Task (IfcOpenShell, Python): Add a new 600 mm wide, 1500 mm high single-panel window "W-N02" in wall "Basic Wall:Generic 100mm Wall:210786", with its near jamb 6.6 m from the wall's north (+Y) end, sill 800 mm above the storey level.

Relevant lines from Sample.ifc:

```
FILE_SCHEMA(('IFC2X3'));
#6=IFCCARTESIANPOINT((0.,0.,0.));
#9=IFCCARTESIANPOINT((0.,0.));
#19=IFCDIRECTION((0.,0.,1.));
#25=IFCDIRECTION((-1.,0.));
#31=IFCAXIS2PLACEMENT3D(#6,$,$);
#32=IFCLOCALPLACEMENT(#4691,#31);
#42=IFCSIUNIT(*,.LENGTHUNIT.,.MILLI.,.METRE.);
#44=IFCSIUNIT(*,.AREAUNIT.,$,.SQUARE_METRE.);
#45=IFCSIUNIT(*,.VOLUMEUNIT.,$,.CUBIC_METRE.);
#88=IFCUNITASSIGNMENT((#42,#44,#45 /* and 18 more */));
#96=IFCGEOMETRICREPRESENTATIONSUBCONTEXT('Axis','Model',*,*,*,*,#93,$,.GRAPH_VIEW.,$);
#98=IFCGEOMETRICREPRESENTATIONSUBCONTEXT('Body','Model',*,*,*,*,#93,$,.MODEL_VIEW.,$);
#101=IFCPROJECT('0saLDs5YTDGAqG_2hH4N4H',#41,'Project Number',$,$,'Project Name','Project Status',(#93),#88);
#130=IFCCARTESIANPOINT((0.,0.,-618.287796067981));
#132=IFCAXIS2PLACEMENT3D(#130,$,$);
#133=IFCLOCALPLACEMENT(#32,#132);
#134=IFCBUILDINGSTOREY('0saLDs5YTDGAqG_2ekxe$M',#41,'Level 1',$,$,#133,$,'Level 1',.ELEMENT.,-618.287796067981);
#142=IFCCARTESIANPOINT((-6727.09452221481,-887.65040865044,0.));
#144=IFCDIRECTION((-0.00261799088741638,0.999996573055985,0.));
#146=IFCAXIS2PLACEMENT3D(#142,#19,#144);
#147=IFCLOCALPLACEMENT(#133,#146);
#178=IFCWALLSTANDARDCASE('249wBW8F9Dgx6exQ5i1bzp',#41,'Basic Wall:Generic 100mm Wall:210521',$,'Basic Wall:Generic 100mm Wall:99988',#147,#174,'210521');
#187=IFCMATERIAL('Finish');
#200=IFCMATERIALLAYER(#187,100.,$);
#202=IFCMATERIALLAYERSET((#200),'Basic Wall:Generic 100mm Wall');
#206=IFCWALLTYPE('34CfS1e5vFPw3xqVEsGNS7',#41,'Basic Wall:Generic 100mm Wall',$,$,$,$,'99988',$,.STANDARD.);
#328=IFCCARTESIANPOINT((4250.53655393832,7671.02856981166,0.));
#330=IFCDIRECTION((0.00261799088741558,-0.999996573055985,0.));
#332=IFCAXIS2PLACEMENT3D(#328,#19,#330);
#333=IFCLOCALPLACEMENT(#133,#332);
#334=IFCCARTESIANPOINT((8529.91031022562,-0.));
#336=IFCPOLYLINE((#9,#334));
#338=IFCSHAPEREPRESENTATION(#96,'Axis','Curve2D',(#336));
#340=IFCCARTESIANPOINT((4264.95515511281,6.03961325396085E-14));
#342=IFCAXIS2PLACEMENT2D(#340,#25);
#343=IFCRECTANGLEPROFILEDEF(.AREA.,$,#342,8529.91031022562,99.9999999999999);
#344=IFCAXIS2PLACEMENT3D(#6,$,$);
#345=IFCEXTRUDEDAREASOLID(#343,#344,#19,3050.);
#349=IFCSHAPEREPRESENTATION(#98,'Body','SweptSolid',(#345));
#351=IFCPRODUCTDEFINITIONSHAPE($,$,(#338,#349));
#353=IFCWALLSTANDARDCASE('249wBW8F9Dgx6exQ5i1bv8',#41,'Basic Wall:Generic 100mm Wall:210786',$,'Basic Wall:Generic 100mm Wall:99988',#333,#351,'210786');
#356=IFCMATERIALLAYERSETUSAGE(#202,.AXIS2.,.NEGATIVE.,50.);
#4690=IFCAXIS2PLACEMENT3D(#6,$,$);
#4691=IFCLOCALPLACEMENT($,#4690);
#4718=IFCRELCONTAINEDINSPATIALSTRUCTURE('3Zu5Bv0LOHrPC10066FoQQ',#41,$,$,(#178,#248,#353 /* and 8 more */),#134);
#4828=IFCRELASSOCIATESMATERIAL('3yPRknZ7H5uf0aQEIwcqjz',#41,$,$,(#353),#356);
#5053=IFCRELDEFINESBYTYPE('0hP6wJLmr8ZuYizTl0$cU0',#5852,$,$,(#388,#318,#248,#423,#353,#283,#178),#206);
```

```python
import numpy as np
import ifcopenshell
import ifcopenshell.api.feature
import ifcopenshell.api.geometry
import ifcopenshell.api.root
import ifcopenshell.api.spatial
import ifcopenshell.api.type
import ifcopenshell.geom
import ifcopenshell.util.element
import ifcopenshell.util.placement
import ifcopenshell.util.representation
import ifcopenshell.util.shape
import ifcopenshell.util.unit

model = ifcopenshell.open("Sample.ifc")
unit_scale = ifcopenshell.util.unit.calculate_unit_scale(model)
settings = ifcopenshell.geom.settings()


def volume(element):
    """Net volume in cubic metres, openings subtracted."""
    shape = ifcopenshell.geom.create_shape(settings, element)
    return ifcopenshell.util.shape.get_volume(shape.geometry)


wall = model.by_id(353)
storey = ifcopenshell.util.element.get_container(wall, ifc_class="IfcBuildingStorey")
context = ifcopenshell.util.representation.get_context(model, "Model", "Body", "MODEL_VIEW")
before = volume(wall)

width, height, from_end, sill = 0.6, 1.5, 6.6, 0.8  # metres

# The wall runs along its own X axis, and the end named is its -X end.
wall_shape = ifcopenshell.geom.create_shape(settings, wall)
x, y, z = ifcopenshell.util.shape.get_vertices(wall_shape.geometry).T
start = x.min() + from_end
face, thickness = float(y.min()), float(y.max() - y.min())
wall_matrix = ifcopenshell.util.placement.get_local_placement(wall.ObjectPlacement)
level = ifcopenshell.util.placement.get_local_placement(storey.ObjectPlacement)[2, 3]


def in_wall(x, y):
    """Placement at x, y metres in the wall's axes, at sill height."""
    matrix = wall_matrix.copy()
    matrix[:, 3] = wall_matrix @ np.array([x / unit_scale, y / unit_scale, 0.0, 1.0])
    matrix[2, 3] = level + sill / unit_scale
    return matrix


# Opening: a box that overshoots both wall faces by 50 mm.
opening = ifcopenshell.api.root.create_entity(model, ifc_class="IfcOpeningElement")
box = ifcopenshell.api.geometry.add_wall_representation(
    model, context=context, length=width, height=height, thickness=thickness + 0.1
)
ifcopenshell.api.geometry.assign_representation(model, product=opening, representation=box)
ifcopenshell.api.geometry.edit_object_placement(model, product=opening, matrix=in_wall(start, face - 0.05), is_si=False)
ifcopenshell.api.feature.add_feature(model, feature=opening, element=wall)

window = ifcopenshell.api.root.create_entity(model, ifc_class="IfcWindow", name="W-N02")
window.OverallWidth, window.OverallHeight = width / unit_scale, height / unit_scale
body = ifcopenshell.api.geometry.add_window_representation(
    model,
    context=context,
    overall_width=window.OverallWidth,
    overall_height=window.OverallHeight,
    partition_type="SINGLE_PANEL",
)
ifcopenshell.api.geometry.assign_representation(model, product=window, representation=body)
ifcopenshell.api.spatial.assign_container(model, products=[window], relating_structure=storey)
fills = ifcopenshell.api.feature.add_filling(model, opening=opening, element=window)
fills.OwnerHistory = window.OwnerHistory  # required in IFC2X3

# IFC2X3 keeps the operation on the window style.
style = ifcopenshell.api.root.create_entity(model, ifc_class="IfcWindowStyle", name="W-N02")
style.OperationType, style.ConstructionType = "SINGLE_PANEL", "NOTDEFINED"
style.ParameterTakesPrecedence = style.Sizeable = False
ifcopenshell.api.type.assign_type(model, related_objects=[window], relating_type=style)

# Centre the window in the wall's thickness.
ifcopenshell.api.geometry.edit_object_placement(model, product=window, matrix=in_wall(start, face), is_si=False)
window_shape = ifcopenshell.geom.create_shape(settings, window)
depth = ifcopenshell.util.shape.get_vertices(window_shape.geometry)[:, 1]
offset = face + thickness / 2 - (depth.min() + depth.max()) / 2
ifcopenshell.api.geometry.edit_object_placement(model, product=window, matrix=in_wall(start, offset), is_si=False)

after = volume(wall)

print(f"wall volume {before:.3f} -> {after:.3f} m3")

model.write("Sample_rev.ifc")
```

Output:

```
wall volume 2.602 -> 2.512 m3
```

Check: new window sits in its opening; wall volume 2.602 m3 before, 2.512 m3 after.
